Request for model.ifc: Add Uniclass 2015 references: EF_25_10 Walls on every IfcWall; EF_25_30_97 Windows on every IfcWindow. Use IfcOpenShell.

First a look at what the model holds.

```python
import ifcopenshell

model = ifcopenshell.open("model.ifc")
print(model.schema)
print("classifications:", [c.Name for c in model.by_type("IfcClassification")])
for ifc_class in ("IfcDoor", "IfcRoof", "IfcStair", "IfcWall", "IfcWindow"):
    print(ifc_class, len(model.by_type(ifc_class)))
```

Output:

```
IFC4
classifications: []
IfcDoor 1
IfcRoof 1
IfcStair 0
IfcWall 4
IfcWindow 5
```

```python
import ifcopenshell
import ifcopenshell.api.classification

model = ifcopenshell.open("model.ifc")

system = ifcopenshell.api.classification.add_classification(model, classification="Uniclass 2015")

codes = {
    "IfcWall": ("EF_25_10", "Walls"),
    "IfcWindow": ("EF_25_30_97", "Windows"),
}
for ifc_class, (code, name) in codes.items():
    products = model.by_type(ifc_class)
    ifcopenshell.api.classification.add_reference(
        model, products=products, classification=system, identification=code, name=name
    )
    print(code, len(products))

model.write("model-out.ifc")
```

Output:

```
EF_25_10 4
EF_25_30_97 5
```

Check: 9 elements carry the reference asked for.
